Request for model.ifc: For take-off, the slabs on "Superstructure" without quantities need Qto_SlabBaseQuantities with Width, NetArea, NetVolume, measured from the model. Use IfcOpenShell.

First a look at what the model holds.

```python
import ifcopenshell
import ifcopenshell.util.element
import ifcopenshell.util.unit

model = ifcopenshell.open("model.ifc")
print(model.schema)
for unit_type in ("LENGTHUNIT", "AREAUNIT", "VOLUMEUNIT"):
    print(unit_type, ifcopenshell.util.unit.calculate_unit_scale(model, unit_type))
storey = next(s for s in model.by_type("IfcBuildingStorey") if s.Name == "Superstructure")
slabs = [e for e in ifcopenshell.util.element.get_decomposition(storey) if e.is_a("IfcSlab")]
for e in sorted(slabs, key=lambda e: e.id()):
    print(e.id(), e.is_a(), e.Name, list(ifcopenshell.util.element.get_psets(e, qtos_only=True)), sep=" | ")
```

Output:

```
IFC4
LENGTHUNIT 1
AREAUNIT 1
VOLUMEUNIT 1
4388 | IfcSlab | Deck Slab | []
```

```python
import ifcopenshell
import ifcopenshell.api.pset
import ifcopenshell.geom
import ifcopenshell.util.element
import ifcopenshell.util.shape
import ifcopenshell.util.unit

model = ifcopenshell.open("model.ifc")
unit_scale = ifcopenshell.util.unit.calculate_unit_scale(model)
area_scale = ifcopenshell.util.unit.calculate_unit_scale(model, "AREAUNIT")
volume_scale = ifcopenshell.util.unit.calculate_unit_scale(model, "VOLUMEUNIT")
settings = ifcopenshell.geom.settings()

storey = next(s for s in model.by_type("IfcBuildingStorey") if s.Name == "Superstructure")
slabs = [e for e in ifcopenshell.util.element.get_decomposition(storey) if e.is_a("IfcSlab")]

for e in sorted(slabs, key=lambda e: e.id()):
    if ifcopenshell.util.element.get_psets(e, qtos_only=True, should_inherit=False):
        continue
    # Geometry comes back in metres, in the element's own axes.
    shape = ifcopenshell.geom.create_shape(settings, e)
    values = {
        "Width": ifcopenshell.util.shape.get_z(shape.geometry) / unit_scale,
        "NetArea": ifcopenshell.util.shape.get_footprint_area(shape.geometry) / area_scale,
        "NetVolume": ifcopenshell.util.shape.get_volume(shape.geometry) / volume_scale,
    }
    qto = ifcopenshell.api.pset.add_qto(model, product=e, name="Qto_SlabBaseQuantities")
    ifcopenshell.api.pset.edit_qto(model, qto=qto, properties=values)
    print(e.id(), {k: round(v, 3) for k, v in values.items()})

model.write("model_rev.ifc")
```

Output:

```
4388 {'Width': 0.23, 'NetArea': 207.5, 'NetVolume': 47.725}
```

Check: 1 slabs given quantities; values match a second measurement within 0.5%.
